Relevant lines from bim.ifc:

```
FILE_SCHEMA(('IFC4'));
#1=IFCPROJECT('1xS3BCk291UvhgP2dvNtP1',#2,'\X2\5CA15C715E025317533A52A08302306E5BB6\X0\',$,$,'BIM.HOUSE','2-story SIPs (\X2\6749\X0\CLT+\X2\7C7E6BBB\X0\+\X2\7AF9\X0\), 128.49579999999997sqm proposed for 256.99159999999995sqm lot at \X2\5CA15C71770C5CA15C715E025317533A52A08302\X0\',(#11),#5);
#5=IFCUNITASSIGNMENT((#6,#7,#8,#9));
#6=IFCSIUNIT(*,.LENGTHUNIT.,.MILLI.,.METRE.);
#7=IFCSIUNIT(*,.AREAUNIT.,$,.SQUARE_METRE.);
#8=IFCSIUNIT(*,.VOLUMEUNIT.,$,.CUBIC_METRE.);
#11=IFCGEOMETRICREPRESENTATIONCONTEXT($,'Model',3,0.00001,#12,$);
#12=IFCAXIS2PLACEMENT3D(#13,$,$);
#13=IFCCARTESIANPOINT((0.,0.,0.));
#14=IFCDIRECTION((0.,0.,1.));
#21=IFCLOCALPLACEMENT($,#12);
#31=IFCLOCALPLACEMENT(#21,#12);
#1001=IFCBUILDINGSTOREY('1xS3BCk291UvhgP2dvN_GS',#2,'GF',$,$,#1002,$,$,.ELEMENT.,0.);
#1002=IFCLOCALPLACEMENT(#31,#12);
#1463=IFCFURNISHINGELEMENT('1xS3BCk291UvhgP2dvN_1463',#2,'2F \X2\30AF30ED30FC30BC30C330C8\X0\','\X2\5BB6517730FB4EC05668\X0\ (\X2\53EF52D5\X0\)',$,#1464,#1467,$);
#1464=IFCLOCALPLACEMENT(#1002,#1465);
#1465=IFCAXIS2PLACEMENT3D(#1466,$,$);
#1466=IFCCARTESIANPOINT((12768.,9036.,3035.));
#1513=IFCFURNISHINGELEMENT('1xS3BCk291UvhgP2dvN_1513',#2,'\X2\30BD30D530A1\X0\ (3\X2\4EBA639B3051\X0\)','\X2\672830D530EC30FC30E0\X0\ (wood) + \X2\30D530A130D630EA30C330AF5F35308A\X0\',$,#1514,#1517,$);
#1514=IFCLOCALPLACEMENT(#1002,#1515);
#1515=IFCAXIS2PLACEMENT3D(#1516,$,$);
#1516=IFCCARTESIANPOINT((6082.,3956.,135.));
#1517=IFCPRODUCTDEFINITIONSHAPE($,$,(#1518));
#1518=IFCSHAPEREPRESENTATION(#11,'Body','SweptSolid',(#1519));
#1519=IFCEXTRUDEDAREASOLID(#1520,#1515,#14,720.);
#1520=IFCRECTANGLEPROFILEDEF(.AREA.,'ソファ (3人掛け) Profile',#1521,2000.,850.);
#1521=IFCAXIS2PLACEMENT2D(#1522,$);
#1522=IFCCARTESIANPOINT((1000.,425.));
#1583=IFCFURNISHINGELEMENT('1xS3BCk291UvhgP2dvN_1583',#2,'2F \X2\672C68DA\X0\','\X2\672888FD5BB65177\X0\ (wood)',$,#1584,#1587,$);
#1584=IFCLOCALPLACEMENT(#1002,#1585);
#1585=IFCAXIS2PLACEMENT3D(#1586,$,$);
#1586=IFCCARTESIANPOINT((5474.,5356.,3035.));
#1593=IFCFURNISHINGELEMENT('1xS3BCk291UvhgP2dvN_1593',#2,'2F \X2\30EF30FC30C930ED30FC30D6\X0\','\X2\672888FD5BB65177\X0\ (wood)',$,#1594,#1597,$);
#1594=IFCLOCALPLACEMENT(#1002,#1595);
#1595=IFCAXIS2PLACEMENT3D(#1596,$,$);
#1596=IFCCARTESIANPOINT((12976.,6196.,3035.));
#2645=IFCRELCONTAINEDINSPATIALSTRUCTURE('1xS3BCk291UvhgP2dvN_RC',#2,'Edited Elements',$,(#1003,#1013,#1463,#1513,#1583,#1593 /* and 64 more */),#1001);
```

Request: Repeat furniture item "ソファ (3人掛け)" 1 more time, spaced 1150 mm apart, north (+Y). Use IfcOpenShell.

```python
import numpy as np
import ifcopenshell
import ifcopenshell.api.geometry
import ifcopenshell.api.root
import ifcopenshell.util.element
import ifcopenshell.util.placement

model = ifcopenshell.open("bim.ifc")


def reuse_history(source, copy):
    """copy_class also copies each property set's owner history, people and application; keep the originals."""
    for rel in copy.IsDefinedBy:
        if rel.is_a("IfcRelDefinesByProperties") and (history := rel.RelatingPropertyDefinition.OwnerHistory):
            rel.RelatingPropertyDefinition.OwnerHistory = source.OwnerHistory
            ifcopenshell.util.element.remove_deep2(model, history)


source = model.by_guid("1xS3BCk291UvhgP2dvN_1513")
base = ifcopenshell.util.placement.get_local_placement(source.ObjectPlacement)
step = np.array([0.0, 1.0, 0.0]) * 1150.0

for i in range(1, 2):
    copy = ifcopenshell.api.root.copy_class(model, product=source)
    copy.Representation = ifcopenshell.util.element.copy_deep(
        model, source.Representation, exclude=["IfcGeometricRepresentationContext", "IfcRepresentationMap"]
    )
    reuse_history(source, copy)
    matrix = base.copy()
    matrix[:3, 3] += i * step
    print("added at", matrix[:3, 3].round(3) + 0.0)
    ifcopenshell.api.geometry.edit_object_placement(model, product=copy, matrix=matrix, is_si=False)

model.write("bim_updated.ifc")
```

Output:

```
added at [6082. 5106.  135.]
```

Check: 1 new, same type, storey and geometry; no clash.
